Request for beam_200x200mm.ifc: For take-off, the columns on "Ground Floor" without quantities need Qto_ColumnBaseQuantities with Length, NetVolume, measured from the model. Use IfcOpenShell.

First a look at what the model holds.

```python
import ifcopenshell
import ifcopenshell.util.element
import ifcopenshell.util.unit

model = ifcopenshell.open("beam_200x200mm.ifc")
print(model.schema)
for unit_type in ("LENGTHUNIT", "AREAUNIT", "VOLUMEUNIT"):
    print(unit_type, ifcopenshell.util.unit.calculate_unit_scale(model, unit_type))
storey = next(s for s in model.by_type("IfcBuildingStorey") if s.Name == "Ground Floor")
columns = [e for e in ifcopenshell.util.element.get_decomposition(storey) if e.is_a("IfcColumn")]
for e in sorted(columns, key=lambda e: e.id()):
    print(e.id(), e.is_a(), e.Name, list(ifcopenshell.util.element.get_psets(e, qtos_only=True)), sep=" | ")
```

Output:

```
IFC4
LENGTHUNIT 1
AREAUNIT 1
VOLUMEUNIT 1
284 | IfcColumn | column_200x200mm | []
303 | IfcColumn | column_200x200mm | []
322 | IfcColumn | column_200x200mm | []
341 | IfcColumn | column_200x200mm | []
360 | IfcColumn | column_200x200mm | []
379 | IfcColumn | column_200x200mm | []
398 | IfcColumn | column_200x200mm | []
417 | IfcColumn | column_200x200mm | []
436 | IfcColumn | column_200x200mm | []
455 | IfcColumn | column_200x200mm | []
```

```python
import ifcopenshell
import ifcopenshell.api.pset
import ifcopenshell.geom
import ifcopenshell.util.element
import ifcopenshell.util.shape
import ifcopenshell.util.unit

model = ifcopenshell.open("beam_200x200mm.ifc")
unit_scale = ifcopenshell.util.unit.calculate_unit_scale(model)
volume_scale = ifcopenshell.util.unit.calculate_unit_scale(model, "VOLUMEUNIT")
settings = ifcopenshell.geom.settings()

storey = next(s for s in model.by_type("IfcBuildingStorey") if s.Name == "Ground Floor")
columns = [e for e in ifcopenshell.util.element.get_decomposition(storey) if e.is_a("IfcColumn")]

for e in sorted(columns, key=lambda e: e.id()):
    if ifcopenshell.util.element.get_psets(e, qtos_only=True, should_inherit=False):
        continue
    # Geometry comes back in metres, in the element's own axes.
    shape = ifcopenshell.geom.create_shape(settings, e)
    values = {
        "Length": ifcopenshell.util.shape.get_z(shape.geometry) / unit_scale,
        "NetVolume": ifcopenshell.util.shape.get_volume(shape.geometry) / volume_scale,
    }
    qto = ifcopenshell.api.pset.add_qto(model, product=e, name="Qto_ColumnBaseQuantities")
    ifcopenshell.api.pset.edit_qto(model, qto=qto, properties=values)
    print(e.id(), {k: round(v, 3) for k, v in values.items()})

model.write("beam_200x200mm_rev.ifc")
```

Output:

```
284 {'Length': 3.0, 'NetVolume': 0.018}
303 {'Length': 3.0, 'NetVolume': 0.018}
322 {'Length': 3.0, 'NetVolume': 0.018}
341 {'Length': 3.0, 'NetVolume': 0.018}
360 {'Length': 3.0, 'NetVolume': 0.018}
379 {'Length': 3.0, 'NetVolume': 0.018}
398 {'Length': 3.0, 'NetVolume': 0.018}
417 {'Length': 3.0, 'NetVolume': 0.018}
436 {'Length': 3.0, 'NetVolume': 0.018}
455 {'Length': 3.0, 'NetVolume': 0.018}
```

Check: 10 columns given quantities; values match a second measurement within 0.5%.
